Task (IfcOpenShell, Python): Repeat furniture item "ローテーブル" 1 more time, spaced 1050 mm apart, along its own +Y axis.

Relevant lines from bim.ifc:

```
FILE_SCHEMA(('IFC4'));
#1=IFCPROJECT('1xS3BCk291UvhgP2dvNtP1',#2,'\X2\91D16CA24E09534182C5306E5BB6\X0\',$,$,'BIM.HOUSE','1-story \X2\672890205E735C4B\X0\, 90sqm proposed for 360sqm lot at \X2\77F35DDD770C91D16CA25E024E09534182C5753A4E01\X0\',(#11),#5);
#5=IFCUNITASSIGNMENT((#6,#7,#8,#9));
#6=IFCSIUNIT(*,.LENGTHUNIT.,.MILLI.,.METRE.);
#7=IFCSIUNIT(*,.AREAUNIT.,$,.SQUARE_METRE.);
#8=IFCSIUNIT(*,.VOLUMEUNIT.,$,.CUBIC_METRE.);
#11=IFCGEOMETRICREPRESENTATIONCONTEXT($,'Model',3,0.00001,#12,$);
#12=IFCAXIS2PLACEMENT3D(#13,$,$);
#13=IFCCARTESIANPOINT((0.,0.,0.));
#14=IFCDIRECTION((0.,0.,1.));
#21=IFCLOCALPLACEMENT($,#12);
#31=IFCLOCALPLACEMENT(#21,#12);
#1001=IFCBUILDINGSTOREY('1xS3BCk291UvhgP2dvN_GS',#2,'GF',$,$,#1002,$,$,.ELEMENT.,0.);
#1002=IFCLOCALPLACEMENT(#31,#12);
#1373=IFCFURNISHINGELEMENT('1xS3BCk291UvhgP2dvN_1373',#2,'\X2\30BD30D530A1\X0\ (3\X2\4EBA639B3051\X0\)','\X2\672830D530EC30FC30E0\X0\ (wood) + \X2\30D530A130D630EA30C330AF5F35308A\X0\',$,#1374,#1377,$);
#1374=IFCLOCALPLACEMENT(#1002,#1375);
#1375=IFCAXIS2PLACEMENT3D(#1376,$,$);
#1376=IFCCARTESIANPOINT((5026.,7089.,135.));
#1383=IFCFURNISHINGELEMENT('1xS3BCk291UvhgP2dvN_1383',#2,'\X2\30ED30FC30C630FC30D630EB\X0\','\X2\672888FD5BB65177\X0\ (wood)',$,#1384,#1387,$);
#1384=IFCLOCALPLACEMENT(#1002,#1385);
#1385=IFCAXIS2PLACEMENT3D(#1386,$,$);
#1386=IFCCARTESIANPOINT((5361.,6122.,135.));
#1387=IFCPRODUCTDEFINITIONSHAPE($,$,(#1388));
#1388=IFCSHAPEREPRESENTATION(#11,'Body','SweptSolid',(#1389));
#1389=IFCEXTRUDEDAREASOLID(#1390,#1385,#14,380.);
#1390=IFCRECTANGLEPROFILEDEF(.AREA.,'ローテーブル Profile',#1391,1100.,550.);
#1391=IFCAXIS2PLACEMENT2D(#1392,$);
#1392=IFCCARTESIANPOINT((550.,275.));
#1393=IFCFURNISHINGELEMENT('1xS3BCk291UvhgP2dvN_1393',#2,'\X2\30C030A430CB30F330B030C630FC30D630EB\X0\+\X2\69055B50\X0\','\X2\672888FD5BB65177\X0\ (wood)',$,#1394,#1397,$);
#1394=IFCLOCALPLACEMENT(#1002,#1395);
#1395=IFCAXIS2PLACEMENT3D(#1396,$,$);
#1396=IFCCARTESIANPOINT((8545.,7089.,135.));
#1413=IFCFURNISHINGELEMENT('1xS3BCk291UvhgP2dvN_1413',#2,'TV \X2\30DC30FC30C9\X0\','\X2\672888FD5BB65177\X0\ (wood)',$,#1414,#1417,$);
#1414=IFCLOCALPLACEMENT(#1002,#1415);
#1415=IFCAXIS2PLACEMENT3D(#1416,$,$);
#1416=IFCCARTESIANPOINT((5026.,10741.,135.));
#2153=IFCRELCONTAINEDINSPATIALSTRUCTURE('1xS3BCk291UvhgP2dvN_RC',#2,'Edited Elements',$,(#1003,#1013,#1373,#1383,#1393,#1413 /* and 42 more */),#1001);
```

```python
import ifcopenshell
import ifcopenshell.api.geometry
import ifcopenshell.api.root
import ifcopenshell.util.element
import ifcopenshell.util.placement
import ifcopenshell.util.unit

model = ifcopenshell.open("bim.ifc")
unit_scale = ifcopenshell.util.unit.calculate_unit_scale(model)


def reuse_history(source, copy):
    """copy_class also copies each property set's owner history, people and application; keep the originals."""
    for rel in copy.IsDefinedBy:
        if rel.is_a("IfcRelDefinesByProperties") and (history := rel.RelatingPropertyDefinition.OwnerHistory):
            rel.RelatingPropertyDefinition.OwnerHistory = source.OwnerHistory
            ifcopenshell.util.element.remove_deep2(model, history)


source = model.by_id(1383)
base = ifcopenshell.util.placement.get_local_placement(source.ObjectPlacement)
step = base[:3, 1] * 1.05 / unit_scale

for i in range(1, 2):
    copy = ifcopenshell.api.root.copy_class(model, product=source)
    copy.Representation = ifcopenshell.util.element.copy_deep(
        model, source.Representation, exclude=["IfcGeometricRepresentationContext", "IfcRepresentationMap"]
    )
    reuse_history(source, copy)
    matrix = base.copy()
    matrix[:3, 3] += i * step
    print("added at", matrix[:3, 3].round(3) + 0.0)
    ifcopenshell.api.geometry.edit_object_placement(model, product=copy, matrix=matrix, is_si=False)

model.write("bim_rev.ifc")
```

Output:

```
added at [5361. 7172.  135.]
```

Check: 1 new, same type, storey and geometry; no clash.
